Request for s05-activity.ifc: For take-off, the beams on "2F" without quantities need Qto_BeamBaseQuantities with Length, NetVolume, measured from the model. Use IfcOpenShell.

First a look at what the model holds.

```python
import ifcopenshell
import ifcopenshell.util.element
import ifcopenshell.util.unit

model = ifcopenshell.open("s05-activity.ifc")
print(model.schema)
for unit_type in ("LENGTHUNIT", "AREAUNIT", "VOLUMEUNIT"):
    print(unit_type, ifcopenshell.util.unit.calculate_unit_scale(model, unit_type))
storey = next(s for s in model.by_type("IfcBuildingStorey") if s.Name == "2F")
beams = [e for e in ifcopenshell.util.element.get_decomposition(storey) if e.is_a("IfcBeam")]
for e in sorted(beams, key=lambda e: e.id()):
    print(e.id(), e.is_a(), e.Name, list(ifcopenshell.util.element.get_psets(e, qtos_only=True)), sep=" | ")
```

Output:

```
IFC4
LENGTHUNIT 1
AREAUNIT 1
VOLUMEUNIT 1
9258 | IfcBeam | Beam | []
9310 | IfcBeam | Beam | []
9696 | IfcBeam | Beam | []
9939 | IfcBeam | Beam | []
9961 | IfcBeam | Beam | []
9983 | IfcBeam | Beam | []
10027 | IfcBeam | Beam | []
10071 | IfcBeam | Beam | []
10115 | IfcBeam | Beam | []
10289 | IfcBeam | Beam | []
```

```python
import ifcopenshell
import ifcopenshell.api.pset
import ifcopenshell.geom
import ifcopenshell.util.element
import ifcopenshell.util.shape
import ifcopenshell.util.unit

model = ifcopenshell.open("s05-activity.ifc")
unit_scale = ifcopenshell.util.unit.calculate_unit_scale(model)
volume_scale = ifcopenshell.util.unit.calculate_unit_scale(model, "VOLUMEUNIT")
settings = ifcopenshell.geom.settings()

storey = next(s for s in model.by_type("IfcBuildingStorey") if s.Name == "2F")
beams = [e for e in ifcopenshell.util.element.get_decomposition(storey) if e.is_a("IfcBeam")]

for e in sorted(beams, key=lambda e: e.id()):
    if ifcopenshell.util.element.get_psets(e, qtos_only=True, should_inherit=False):
        continue
    # Geometry comes back in metres, in the element's own axes.
    shape = ifcopenshell.geom.create_shape(settings, e)
    values = {
        "Length": ifcopenshell.util.shape.get_max_xyz(shape.geometry) / unit_scale,
        "NetVolume": ifcopenshell.util.shape.get_volume(shape.geometry) / volume_scale,
    }
    qto = ifcopenshell.api.pset.add_qto(model, product=e, name="Qto_BeamBaseQuantities")
    ifcopenshell.api.pset.edit_qto(model, qto=qto, properties=values)
    print(e.id(), {k: round(v, 3) for k, v in values.items()})

model.write("s05-activity-out.ifc")
```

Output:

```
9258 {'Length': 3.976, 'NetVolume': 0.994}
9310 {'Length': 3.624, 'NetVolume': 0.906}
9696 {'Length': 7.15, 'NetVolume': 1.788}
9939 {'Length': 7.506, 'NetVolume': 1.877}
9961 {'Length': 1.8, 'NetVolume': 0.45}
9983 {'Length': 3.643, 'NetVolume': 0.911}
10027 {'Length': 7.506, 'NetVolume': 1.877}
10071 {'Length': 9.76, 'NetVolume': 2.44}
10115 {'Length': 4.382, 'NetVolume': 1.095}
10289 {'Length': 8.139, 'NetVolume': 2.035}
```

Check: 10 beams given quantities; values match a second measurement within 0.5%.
